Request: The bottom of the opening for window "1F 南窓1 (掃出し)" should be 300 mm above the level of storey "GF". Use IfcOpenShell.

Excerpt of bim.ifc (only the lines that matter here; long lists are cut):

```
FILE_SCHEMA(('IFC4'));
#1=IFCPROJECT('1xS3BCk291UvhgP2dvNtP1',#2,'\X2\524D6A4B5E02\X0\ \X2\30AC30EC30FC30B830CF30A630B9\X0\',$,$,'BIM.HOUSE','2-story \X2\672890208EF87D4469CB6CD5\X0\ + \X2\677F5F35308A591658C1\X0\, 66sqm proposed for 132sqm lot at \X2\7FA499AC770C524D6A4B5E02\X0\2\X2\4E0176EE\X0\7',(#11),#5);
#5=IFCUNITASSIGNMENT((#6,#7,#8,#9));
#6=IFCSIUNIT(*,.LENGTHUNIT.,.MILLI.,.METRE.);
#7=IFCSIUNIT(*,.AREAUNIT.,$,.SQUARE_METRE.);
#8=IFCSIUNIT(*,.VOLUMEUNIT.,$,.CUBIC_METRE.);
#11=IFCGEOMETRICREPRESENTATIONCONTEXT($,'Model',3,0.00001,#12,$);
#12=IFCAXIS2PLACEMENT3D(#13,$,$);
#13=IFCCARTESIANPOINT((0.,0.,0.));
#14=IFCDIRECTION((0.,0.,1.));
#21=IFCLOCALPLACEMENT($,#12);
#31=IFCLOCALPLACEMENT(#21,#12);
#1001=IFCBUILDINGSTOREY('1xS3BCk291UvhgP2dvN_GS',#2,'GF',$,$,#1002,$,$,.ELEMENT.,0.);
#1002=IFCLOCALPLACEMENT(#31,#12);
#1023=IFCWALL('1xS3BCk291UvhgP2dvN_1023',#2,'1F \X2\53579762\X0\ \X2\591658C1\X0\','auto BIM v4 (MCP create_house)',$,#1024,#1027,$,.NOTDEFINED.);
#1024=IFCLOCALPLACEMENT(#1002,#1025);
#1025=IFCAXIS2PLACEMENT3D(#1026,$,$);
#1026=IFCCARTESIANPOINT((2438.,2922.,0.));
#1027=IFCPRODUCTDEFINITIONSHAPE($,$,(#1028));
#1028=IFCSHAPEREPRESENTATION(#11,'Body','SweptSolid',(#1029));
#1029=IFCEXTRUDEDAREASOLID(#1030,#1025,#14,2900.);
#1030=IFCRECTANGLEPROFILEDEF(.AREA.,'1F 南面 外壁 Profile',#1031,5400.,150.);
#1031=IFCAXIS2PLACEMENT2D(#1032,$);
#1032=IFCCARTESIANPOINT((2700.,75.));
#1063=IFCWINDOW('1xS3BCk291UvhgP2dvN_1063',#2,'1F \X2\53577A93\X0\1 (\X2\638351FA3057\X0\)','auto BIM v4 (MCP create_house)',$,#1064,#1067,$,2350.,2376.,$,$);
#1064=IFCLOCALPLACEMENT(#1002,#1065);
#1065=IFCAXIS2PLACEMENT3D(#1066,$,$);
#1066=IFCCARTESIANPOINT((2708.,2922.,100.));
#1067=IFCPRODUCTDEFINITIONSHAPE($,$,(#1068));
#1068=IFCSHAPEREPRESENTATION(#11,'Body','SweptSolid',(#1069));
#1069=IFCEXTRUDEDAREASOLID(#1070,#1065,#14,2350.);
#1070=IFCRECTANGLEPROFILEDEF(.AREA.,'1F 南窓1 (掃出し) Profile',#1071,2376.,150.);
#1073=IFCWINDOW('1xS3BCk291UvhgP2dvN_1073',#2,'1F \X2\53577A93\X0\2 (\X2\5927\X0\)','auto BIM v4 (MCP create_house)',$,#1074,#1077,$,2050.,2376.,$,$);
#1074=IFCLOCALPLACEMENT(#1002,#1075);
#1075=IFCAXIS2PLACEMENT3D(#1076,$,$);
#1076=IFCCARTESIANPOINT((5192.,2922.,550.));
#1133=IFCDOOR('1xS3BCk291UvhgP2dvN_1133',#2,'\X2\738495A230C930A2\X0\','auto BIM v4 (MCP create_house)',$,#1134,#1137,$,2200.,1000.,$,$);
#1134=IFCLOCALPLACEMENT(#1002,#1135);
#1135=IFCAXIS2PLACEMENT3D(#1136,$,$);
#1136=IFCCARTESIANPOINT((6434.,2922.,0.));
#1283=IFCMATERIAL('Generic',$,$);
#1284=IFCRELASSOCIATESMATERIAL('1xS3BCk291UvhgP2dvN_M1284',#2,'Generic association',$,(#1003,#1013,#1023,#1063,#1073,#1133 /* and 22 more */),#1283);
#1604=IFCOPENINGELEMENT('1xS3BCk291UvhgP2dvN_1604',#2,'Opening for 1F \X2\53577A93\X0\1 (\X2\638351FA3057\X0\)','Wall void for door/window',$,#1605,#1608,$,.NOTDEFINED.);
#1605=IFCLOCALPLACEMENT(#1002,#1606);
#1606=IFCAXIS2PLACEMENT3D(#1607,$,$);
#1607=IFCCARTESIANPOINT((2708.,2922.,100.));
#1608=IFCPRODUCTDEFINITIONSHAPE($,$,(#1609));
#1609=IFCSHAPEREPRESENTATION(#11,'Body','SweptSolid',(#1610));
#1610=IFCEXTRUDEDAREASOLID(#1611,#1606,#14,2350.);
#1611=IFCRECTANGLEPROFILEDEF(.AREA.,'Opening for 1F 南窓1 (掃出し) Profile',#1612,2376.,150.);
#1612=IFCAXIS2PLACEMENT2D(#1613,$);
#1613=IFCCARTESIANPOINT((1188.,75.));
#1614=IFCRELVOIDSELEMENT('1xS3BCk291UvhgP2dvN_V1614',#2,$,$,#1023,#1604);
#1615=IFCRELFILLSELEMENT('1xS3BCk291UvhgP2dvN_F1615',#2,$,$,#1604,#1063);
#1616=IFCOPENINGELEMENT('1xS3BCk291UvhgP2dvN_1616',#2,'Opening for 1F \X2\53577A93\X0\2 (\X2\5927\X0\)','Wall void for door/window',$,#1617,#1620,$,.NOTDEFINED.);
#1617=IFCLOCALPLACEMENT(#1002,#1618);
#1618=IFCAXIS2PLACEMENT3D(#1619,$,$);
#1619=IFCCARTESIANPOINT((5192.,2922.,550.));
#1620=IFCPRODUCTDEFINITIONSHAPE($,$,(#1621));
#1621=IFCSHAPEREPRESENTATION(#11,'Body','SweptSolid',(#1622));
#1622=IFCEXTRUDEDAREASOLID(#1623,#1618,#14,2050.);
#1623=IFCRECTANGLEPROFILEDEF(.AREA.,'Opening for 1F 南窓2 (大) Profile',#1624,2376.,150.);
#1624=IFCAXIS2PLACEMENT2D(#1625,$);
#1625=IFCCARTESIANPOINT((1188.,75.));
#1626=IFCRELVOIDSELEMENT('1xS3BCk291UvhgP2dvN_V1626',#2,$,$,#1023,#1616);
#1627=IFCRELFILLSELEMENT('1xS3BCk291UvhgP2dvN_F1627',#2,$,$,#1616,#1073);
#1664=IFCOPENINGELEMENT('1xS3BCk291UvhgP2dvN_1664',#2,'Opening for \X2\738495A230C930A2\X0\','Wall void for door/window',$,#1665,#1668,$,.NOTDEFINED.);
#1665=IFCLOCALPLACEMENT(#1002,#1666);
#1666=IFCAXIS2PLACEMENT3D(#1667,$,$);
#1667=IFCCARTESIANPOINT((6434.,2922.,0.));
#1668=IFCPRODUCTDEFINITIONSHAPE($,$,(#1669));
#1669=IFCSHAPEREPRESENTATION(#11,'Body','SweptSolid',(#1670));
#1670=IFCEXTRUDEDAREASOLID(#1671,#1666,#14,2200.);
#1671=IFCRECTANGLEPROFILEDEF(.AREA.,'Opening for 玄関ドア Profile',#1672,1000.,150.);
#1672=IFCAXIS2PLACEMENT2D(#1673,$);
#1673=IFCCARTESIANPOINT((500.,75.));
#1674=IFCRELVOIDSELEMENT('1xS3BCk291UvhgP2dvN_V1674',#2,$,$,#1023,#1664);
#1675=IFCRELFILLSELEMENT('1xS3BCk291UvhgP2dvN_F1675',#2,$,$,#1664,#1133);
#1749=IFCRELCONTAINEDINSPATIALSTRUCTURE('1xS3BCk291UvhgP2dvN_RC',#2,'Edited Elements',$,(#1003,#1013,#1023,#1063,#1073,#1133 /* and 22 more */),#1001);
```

```python
import numpy as np
import ifcopenshell
import ifcopenshell.api.geometry
import ifcopenshell.geom
import ifcopenshell.util.element
import ifcopenshell.util.placement
import ifcopenshell.util.shape
import ifcopenshell.util.unit

model = ifcopenshell.open("bim.ifc")
unit_scale = ifcopenshell.util.unit.calculate_unit_scale(model)

window = model.by_guid("1xS3BCk291UvhgP2dvN_1063")
opening = window.FillsVoids[0].RelatingOpeningElement
storey = ifcopenshell.util.element.get_container(window, ifc_class="IfcBuildingStorey")
level = ifcopenshell.util.placement.get_local_placement(storey.ObjectPlacement)[2, 3]

# The opening's origin need not be at the sill, so measure its lowest point.
shape = ifcopenshell.geom.create_shape(ifcopenshell.geom.settings(), opening)
bottom = ifcopenshell.util.shape.get_shape_bottom_elevation(shape, shape.geometry) / unit_scale
dz = level + 300.0 - bottom

shift = np.array([0.0, 0.0, dz])
# The window is not placed relative to its opening, so move both.
for product in (opening, window):
    matrix = ifcopenshell.util.placement.get_local_placement(product.ObjectPlacement)
    matrix[:3, 3] += shift
    ifcopenshell.api.geometry.edit_object_placement(model, product=product, matrix=matrix, is_si=False)

print(f"moved by {dz * unit_scale:+.3f} m")

model.write("bim_rev.ifc")
```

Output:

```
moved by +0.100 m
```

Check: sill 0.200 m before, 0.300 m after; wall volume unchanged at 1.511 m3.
